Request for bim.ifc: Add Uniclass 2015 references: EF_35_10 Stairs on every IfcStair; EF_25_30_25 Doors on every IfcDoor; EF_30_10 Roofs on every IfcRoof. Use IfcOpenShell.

First a look at what the model holds.

```python
import ifcopenshell

model = ifcopenshell.open("bim.ifc")
print(model.schema)
print("classifications:", [c.Name for c in model.by_type("IfcClassification")])
for ifc_class in ("IfcDoor", "IfcRoof", "IfcStair", "IfcWall", "IfcWindow"):
    print(ifc_class, len(model.by_type(ifc_class)))
```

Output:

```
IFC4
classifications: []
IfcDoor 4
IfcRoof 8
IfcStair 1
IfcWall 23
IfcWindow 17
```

```python
import ifcopenshell
import ifcopenshell.api.classification

model = ifcopenshell.open("bim.ifc")

system = ifcopenshell.api.classification.add_classification(model, classification="Uniclass 2015")

codes = {
    "IfcStair": ("EF_35_10", "Stairs"),
    "IfcDoor": ("EF_25_30_25", "Doors"),
    "IfcRoof": ("EF_30_10", "Roofs"),
}
for ifc_class, (code, name) in codes.items():
    products = model.by_type(ifc_class)
    ifcopenshell.api.classification.add_reference(
        model, products=products, classification=system, identification=code, name=name
    )
    print(code, len(products))

model.write("bim_v2.ifc")
```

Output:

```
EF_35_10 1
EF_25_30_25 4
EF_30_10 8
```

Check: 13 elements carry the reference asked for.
